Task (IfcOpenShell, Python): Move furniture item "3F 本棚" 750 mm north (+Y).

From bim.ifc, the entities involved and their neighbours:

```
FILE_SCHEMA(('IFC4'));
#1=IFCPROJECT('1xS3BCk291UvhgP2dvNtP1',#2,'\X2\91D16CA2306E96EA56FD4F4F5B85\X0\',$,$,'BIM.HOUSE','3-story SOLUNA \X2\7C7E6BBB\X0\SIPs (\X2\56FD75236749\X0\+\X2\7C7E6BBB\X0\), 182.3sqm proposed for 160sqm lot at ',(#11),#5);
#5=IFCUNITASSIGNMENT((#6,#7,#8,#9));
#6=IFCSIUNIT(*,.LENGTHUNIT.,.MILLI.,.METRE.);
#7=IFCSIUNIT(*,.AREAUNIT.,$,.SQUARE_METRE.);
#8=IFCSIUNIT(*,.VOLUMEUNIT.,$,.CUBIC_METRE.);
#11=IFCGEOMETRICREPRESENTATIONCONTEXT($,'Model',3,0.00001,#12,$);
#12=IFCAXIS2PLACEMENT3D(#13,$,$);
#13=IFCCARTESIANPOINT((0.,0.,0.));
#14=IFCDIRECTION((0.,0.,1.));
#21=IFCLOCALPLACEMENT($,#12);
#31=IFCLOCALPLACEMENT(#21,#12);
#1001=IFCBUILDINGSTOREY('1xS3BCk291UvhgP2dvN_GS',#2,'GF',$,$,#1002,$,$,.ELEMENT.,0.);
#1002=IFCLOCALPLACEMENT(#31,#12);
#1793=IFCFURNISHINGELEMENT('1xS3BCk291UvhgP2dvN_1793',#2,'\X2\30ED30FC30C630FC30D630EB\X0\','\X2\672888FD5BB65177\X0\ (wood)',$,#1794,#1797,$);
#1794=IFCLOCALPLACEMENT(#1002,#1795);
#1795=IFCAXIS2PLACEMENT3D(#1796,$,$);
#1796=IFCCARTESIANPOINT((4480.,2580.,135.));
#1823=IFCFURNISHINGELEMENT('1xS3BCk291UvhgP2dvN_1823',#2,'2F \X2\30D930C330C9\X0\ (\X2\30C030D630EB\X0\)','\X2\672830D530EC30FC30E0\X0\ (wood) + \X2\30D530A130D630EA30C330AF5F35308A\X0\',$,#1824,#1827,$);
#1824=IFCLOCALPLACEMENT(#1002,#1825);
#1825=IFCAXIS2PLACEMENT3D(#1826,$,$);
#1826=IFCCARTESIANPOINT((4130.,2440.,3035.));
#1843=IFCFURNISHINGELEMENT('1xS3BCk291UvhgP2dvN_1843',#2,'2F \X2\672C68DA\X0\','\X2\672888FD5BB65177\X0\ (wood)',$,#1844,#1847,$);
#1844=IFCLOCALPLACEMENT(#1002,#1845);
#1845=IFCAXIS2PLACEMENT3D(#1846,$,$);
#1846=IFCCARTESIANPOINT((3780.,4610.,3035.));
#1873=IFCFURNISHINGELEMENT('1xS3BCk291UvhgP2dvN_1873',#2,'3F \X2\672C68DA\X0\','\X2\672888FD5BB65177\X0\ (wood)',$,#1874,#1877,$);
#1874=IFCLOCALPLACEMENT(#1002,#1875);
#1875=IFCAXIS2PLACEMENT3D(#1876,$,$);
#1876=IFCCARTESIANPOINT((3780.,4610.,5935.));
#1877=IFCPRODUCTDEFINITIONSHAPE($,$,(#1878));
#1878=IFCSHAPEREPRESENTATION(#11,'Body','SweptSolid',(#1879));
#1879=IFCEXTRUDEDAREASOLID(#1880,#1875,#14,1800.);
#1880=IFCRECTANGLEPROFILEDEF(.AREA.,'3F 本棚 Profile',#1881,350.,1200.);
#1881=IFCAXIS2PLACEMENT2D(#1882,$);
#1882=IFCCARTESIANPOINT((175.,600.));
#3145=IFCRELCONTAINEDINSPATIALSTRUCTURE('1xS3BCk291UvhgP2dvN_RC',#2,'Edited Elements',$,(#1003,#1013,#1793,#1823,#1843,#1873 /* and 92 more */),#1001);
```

```python
import ifcopenshell
import ifcopenshell.api.geometry
import ifcopenshell.util.placement
import ifcopenshell.util.unit

model = ifcopenshell.open("bim.ifc")
unit_scale = ifcopenshell.util.unit.calculate_unit_scale(model)

item = model.by_guid("1xS3BCk291UvhgP2dvN_1873")
matrix = ifcopenshell.util.placement.get_local_placement(item.ObjectPlacement)
matrix[1, 3] += 0.75 / unit_scale
ifcopenshell.api.geometry.edit_object_placement(model, product=item, matrix=matrix, is_si=False)

print(ifcopenshell.util.placement.get_local_placement(item.ObjectPlacement).round(3) + 0.0)

model.write("bim-out.ifc")
```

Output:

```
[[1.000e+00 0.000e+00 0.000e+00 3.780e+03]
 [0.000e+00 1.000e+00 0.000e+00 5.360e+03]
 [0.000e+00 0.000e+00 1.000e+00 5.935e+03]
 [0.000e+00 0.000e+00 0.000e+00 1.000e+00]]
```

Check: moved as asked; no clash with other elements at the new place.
